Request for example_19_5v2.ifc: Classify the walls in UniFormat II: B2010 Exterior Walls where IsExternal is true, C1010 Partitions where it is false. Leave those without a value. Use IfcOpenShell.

First a look at what the model holds.

```python
import ifcopenshell
import ifcopenshell.util.element

model = ifcopenshell.open("example_19_5v2.ifc")
print(model.schema)
print("classifications:", [c.Name for c in model.by_type("IfcClassification")])
values = [ifcopenshell.util.element.get_pset(e, "Pset_WallCommon", "IsExternal") for e in model.by_type("IfcWall")]
for value in (True, False, None):
    print("IsExternal", value, values.count(value))
```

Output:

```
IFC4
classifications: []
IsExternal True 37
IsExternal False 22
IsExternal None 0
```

```python
import ifcopenshell
import ifcopenshell.api.classification
import ifcopenshell.util.element

model = ifcopenshell.open("example_19_5v2.ifc")

system = ifcopenshell.api.classification.add_classification(model, classification="UniFormat II")

walls = model.by_type("IfcWall")
external = {e: ifcopenshell.util.element.get_pset(e, "Pset_WallCommon", "IsExternal") for e in walls}
for flag, code, name in ((True, "B2010", "Exterior Walls"), (False, "C1010", "Partitions")):
    products = [e for e in walls if external[e] is flag]
    ifcopenshell.api.classification.add_reference(
        model, products=products, classification=system, identification=code, name=name
    )
    print(code, len(products))

model.write("example_19_5v2-out.ifc")
```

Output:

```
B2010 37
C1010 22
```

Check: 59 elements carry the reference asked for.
